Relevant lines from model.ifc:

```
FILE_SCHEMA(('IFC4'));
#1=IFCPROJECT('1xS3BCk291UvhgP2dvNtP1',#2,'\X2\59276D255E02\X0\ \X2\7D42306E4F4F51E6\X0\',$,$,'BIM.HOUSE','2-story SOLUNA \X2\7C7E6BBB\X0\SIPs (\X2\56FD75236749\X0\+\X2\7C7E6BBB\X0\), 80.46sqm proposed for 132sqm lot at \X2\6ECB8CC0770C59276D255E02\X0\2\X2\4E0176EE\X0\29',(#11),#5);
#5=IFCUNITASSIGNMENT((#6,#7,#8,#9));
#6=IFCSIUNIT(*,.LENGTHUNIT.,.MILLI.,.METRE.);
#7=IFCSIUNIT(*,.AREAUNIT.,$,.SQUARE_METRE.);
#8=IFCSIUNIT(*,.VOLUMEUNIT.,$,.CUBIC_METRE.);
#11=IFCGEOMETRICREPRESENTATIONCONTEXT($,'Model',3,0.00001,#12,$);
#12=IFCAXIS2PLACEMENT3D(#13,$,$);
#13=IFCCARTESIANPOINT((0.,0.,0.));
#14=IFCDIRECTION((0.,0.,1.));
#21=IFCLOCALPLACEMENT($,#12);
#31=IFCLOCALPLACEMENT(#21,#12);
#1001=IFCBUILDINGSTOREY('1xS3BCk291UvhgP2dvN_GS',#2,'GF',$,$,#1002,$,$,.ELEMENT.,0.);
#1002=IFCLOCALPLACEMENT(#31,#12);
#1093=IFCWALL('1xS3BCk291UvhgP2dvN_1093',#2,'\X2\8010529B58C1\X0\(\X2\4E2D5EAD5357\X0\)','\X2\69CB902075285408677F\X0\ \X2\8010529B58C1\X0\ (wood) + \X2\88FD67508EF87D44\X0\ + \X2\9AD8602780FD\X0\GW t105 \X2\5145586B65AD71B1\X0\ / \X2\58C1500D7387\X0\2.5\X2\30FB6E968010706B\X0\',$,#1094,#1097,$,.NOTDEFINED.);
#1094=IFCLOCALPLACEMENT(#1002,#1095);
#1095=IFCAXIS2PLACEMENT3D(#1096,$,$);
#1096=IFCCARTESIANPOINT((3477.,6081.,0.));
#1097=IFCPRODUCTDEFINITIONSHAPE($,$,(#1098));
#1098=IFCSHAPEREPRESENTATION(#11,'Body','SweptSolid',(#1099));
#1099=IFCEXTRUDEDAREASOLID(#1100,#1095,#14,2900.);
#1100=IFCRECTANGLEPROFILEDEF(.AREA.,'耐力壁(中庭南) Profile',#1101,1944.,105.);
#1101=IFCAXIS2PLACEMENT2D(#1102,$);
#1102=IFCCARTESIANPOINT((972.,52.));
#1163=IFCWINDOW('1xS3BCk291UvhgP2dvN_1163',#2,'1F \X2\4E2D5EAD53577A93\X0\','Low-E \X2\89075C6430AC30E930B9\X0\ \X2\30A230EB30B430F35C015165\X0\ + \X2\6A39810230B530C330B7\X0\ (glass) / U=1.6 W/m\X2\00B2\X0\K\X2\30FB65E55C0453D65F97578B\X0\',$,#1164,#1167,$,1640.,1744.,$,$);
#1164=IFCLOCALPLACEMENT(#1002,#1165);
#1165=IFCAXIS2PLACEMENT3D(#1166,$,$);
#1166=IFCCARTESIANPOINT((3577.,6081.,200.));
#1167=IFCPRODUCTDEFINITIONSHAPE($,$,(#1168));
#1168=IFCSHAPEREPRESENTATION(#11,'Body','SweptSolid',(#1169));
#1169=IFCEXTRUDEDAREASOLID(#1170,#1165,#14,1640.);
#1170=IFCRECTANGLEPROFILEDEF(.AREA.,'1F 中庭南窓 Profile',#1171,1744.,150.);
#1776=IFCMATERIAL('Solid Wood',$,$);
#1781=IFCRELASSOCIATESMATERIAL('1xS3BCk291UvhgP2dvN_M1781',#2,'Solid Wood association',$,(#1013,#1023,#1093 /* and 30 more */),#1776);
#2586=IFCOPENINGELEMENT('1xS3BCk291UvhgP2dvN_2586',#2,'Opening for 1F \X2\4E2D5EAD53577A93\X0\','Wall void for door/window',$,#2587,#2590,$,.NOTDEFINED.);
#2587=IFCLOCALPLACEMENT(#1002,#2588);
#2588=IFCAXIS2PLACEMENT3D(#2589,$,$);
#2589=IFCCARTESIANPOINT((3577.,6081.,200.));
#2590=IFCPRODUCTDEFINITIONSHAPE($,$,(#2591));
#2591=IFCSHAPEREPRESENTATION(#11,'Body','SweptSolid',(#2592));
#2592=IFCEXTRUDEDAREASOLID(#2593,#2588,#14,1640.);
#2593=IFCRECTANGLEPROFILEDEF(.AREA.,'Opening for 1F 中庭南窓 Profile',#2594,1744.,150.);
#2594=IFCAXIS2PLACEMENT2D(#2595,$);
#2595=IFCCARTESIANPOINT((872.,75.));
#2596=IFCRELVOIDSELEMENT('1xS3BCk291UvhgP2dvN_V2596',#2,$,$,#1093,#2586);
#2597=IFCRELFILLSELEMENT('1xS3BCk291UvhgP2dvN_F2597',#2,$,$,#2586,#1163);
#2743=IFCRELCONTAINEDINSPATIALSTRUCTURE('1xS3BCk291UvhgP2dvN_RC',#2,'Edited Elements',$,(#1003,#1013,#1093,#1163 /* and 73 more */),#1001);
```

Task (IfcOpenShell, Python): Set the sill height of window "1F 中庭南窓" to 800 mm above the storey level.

```python
import numpy as np
import ifcopenshell
import ifcopenshell.api.geometry
import ifcopenshell.geom
import ifcopenshell.util.element
import ifcopenshell.util.placement
import ifcopenshell.util.shape
import ifcopenshell.util.unit

model = ifcopenshell.open("model.ifc")
unit_scale = ifcopenshell.util.unit.calculate_unit_scale(model)

window = model.by_guid("1xS3BCk291UvhgP2dvN_1163")
opening = window.FillsVoids[0].RelatingOpeningElement
storey = ifcopenshell.util.element.get_container(window, ifc_class="IfcBuildingStorey")
level = ifcopenshell.util.placement.get_local_placement(storey.ObjectPlacement)[2, 3]

# The opening's origin need not be at the sill, so measure its lowest point.
shape = ifcopenshell.geom.create_shape(ifcopenshell.geom.settings(), opening)
bottom = ifcopenshell.util.shape.get_shape_bottom_elevation(shape, shape.geometry) / unit_scale
dz = level + 800.0 - bottom

shift = np.array([0.0, 0.0, dz])
# The window is not placed relative to its opening, so move both.
for product in (opening, window):
    matrix = ifcopenshell.util.placement.get_local_placement(product.ObjectPlacement)
    matrix[:3, 3] += shift
    ifcopenshell.api.geometry.edit_object_placement(model, product=product, matrix=matrix, is_si=False)

print(f"moved by {dz * unit_scale:+.3f} m")

model.write("model_updated.ifc")
```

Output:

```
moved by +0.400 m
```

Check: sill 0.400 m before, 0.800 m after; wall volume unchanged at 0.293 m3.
